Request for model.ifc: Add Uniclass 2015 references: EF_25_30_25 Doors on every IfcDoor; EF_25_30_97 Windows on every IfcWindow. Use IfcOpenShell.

First a look at what the model holds.

```python
import ifcopenshell

model = ifcopenshell.open("model.ifc")
print(model.schema)
print("classifications:", [c.Name for c in model.by_type("IfcClassification")])
for ifc_class in ("IfcDoor", "IfcRoof", "IfcStair", "IfcWall", "IfcWindow"):
    print(ifc_class, len(model.by_type(ifc_class)))
```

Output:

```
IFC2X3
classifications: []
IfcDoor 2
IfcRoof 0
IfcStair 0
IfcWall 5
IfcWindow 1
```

```python
import ifcopenshell
import ifcopenshell.api.classification

model = ifcopenshell.open("model.ifc")

# IFC2X3 requires Source and Edition and has no link from the project to the system.
system = model.create_entity("IfcClassification", Source="NBS", Edition="2015", Name="Uniclass 2015")

codes = {
    "IfcDoor": ("EF_25_30_25", "Doors"),
    "IfcWindow": ("EF_25_30_97", "Windows"),
}
for ifc_class, (code, name) in codes.items():
    products = model.by_type(ifc_class)
    ifcopenshell.api.classification.add_reference(
        model, products=products, classification=system, identification=code, name=name
    )
    print(code, len(products))

model.write("model_updated.ifc")
```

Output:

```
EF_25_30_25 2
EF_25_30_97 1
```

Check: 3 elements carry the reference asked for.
